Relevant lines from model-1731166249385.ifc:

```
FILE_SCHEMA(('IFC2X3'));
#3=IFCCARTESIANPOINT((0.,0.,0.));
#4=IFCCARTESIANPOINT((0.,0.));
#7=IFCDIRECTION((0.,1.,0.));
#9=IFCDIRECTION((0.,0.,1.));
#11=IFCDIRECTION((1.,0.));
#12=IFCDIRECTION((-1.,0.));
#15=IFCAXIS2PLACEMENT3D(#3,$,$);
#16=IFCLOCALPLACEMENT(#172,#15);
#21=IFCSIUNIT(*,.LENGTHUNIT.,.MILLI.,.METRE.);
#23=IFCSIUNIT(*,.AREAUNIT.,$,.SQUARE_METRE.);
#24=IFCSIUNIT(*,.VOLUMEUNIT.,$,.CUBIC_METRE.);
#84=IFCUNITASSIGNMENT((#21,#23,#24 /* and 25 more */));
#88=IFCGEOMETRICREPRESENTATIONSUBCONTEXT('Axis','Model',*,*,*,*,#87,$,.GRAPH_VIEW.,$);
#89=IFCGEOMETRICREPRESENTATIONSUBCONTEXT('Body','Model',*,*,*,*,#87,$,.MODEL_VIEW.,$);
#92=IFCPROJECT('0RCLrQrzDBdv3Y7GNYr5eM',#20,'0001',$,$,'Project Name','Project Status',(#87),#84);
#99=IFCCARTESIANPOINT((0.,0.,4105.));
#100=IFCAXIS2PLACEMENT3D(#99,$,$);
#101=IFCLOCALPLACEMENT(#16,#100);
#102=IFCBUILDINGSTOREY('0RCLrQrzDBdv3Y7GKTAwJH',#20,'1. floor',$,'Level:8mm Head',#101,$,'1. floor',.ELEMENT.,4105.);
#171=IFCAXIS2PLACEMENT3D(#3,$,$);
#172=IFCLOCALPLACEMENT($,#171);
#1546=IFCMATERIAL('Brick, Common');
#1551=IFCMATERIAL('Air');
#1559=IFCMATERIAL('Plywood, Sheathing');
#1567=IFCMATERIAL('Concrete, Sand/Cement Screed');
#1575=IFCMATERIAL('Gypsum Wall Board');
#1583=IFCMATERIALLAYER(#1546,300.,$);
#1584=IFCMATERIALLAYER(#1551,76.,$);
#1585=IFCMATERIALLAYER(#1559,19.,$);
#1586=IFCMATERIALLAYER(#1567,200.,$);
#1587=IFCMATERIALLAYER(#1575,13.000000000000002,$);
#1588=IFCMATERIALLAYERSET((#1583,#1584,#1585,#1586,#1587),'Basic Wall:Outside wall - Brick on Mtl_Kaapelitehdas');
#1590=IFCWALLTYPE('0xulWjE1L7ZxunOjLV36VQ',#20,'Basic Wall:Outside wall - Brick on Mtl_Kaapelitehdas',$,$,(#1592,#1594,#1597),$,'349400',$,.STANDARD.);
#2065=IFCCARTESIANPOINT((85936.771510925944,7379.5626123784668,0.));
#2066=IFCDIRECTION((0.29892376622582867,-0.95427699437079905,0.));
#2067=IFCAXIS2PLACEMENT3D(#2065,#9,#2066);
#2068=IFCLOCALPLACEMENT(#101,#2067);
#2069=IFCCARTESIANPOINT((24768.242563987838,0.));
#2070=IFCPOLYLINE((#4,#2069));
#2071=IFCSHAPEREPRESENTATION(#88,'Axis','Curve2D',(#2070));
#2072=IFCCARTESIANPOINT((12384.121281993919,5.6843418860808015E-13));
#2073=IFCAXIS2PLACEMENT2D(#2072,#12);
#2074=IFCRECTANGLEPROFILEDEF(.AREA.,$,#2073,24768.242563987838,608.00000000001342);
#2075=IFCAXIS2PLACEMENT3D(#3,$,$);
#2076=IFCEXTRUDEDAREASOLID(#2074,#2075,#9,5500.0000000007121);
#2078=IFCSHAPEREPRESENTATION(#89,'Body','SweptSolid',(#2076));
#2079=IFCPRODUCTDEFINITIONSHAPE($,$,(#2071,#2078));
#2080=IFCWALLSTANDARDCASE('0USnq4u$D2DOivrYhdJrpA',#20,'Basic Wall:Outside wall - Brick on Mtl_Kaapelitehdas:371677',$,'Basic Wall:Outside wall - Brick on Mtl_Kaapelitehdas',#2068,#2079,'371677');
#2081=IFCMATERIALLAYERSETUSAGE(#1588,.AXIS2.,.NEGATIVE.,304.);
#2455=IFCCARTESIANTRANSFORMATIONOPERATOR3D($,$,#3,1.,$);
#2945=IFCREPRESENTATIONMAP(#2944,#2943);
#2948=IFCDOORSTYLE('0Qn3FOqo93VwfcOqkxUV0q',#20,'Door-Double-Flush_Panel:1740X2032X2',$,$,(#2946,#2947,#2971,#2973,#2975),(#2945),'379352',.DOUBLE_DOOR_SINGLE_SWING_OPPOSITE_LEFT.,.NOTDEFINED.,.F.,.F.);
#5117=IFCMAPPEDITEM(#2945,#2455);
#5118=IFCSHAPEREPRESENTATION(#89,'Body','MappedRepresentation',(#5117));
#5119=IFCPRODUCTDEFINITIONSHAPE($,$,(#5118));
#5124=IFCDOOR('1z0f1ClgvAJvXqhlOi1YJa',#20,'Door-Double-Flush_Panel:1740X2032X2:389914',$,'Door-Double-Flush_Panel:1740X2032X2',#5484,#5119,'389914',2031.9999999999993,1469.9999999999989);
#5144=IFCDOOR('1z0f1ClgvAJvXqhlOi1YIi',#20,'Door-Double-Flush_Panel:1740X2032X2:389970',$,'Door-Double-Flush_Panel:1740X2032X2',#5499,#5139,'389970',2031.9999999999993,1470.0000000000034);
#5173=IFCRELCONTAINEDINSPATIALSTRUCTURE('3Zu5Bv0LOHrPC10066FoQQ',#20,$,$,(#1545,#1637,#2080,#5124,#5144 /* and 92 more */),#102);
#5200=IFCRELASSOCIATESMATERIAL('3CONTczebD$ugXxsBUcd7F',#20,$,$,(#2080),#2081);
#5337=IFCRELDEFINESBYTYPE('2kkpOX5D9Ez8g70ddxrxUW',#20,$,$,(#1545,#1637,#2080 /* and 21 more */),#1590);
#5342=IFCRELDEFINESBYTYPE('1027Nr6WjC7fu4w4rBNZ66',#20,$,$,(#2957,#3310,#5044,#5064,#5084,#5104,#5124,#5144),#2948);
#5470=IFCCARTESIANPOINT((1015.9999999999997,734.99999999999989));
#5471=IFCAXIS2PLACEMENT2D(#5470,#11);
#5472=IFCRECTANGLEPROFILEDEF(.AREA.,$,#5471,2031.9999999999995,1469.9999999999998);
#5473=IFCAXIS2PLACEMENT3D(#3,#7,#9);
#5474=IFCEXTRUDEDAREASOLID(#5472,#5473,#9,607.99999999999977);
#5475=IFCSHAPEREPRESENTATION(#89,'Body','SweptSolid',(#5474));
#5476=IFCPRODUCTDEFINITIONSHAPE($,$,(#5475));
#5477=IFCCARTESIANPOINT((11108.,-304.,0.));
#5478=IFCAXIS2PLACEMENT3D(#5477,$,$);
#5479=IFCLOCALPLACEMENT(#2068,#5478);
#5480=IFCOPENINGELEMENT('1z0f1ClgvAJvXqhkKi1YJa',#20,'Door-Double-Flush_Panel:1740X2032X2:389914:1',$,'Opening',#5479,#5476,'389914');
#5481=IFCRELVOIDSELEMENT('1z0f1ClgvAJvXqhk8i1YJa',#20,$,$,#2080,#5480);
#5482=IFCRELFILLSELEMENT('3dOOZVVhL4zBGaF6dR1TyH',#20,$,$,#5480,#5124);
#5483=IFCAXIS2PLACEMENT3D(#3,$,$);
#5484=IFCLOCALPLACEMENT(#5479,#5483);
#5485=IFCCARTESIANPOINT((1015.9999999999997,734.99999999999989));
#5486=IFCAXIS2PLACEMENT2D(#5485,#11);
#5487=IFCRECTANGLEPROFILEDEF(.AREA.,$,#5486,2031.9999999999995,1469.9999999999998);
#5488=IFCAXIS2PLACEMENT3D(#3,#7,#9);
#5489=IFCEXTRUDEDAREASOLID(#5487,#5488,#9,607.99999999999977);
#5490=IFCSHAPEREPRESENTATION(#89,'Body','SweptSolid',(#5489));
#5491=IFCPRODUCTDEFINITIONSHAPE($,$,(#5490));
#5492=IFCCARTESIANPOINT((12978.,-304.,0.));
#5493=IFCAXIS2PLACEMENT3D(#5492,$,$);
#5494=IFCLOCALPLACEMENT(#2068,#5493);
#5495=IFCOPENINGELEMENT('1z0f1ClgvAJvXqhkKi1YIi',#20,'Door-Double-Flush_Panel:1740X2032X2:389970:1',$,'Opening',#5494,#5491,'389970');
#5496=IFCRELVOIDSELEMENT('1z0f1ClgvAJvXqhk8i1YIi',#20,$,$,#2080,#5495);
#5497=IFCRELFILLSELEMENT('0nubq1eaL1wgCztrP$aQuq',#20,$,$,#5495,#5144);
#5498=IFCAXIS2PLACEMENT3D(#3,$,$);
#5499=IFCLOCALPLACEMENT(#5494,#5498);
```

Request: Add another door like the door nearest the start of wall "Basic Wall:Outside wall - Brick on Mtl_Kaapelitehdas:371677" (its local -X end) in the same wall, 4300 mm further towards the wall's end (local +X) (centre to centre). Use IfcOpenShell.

```python
import ifcopenshell
import ifcopenshell.api.feature
import ifcopenshell.api.geometry
import ifcopenshell.api.root
import ifcopenshell.geom
import ifcopenshell.util.element
import ifcopenshell.util.placement
import ifcopenshell.util.shape
import ifcopenshell.util.unit

model = ifcopenshell.open("model-1731166249385.ifc")
unit_scale = ifcopenshell.util.unit.calculate_unit_scale(model)
settings = ifcopenshell.geom.settings()


def volume(element):
    """Net volume in cubic metres, openings subtracted."""
    shape = ifcopenshell.geom.create_shape(settings, element)
    return ifcopenshell.util.shape.get_volume(shape.geometry)


def reuse_history(source, copy):
    """copy_class also copies each property set's owner history, people and application; keep the originals."""
    for rel in copy.IsDefinedBy:
        if rel.is_a("IfcRelDefinesByProperties") and (history := rel.RelatingPropertyDefinition.OwnerHistory):
            rel.RelatingPropertyDefinition.OwnerHistory = source.OwnerHistory
            ifcopenshell.util.element.remove_deep2(model, history)


door = model.by_id(5124)
opening = door.FillsVoids[0].RelatingOpeningElement
wall = opening.VoidsElements[0].RelatingBuildingElement
before = volume(wall)
shift = ifcopenshell.util.placement.get_local_placement(wall.ObjectPlacement)[:3, 0] * 4.3 / unit_scale

# copy_class copies the void relationship, type, container and properties, but no geometry.
new_opening = ifcopenshell.api.root.copy_class(model, product=opening)
new_opening.Representation = ifcopenshell.util.element.copy_deep(
    model, opening.Representation, exclude=["IfcGeometricRepresentationContext", "IfcRepresentationMap"]
)
new_opening.Name = "Door-Double-Flush_Panel:1740X2032X2"
new_opening.Tag = None
new_door = ifcopenshell.api.root.copy_class(model, product=door)
new_door.Representation = ifcopenshell.util.element.copy_deep(
    model, door.Representation, exclude=["IfcGeometricRepresentationContext", "IfcRepresentationMap"]
)
new_door.Name = "Door-Double-Flush_Panel:1740X2032X2"
new_door.Tag = None
reuse_history(door, new_door)
fills = ifcopenshell.api.feature.add_filling(model, opening=new_opening, element=new_door)
fills.OwnerHistory = new_door.OwnerHistory  # required in IFC2X3

for old, new in ((opening, new_opening), (door, new_door)):
    matrix = ifcopenshell.util.placement.get_local_placement(old.ObjectPlacement)
    matrix[:3, 3] += shift
    ifcopenshell.api.geometry.edit_object_placement(model, product=new, matrix=matrix, is_si=False)

after = volume(wall)

print(f"wall volume {before:.3f} -> {after:.3f} m3")

model.write("model-1731166249385-out.ifc")
```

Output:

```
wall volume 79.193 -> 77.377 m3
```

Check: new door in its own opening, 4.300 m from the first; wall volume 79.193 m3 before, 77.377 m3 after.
